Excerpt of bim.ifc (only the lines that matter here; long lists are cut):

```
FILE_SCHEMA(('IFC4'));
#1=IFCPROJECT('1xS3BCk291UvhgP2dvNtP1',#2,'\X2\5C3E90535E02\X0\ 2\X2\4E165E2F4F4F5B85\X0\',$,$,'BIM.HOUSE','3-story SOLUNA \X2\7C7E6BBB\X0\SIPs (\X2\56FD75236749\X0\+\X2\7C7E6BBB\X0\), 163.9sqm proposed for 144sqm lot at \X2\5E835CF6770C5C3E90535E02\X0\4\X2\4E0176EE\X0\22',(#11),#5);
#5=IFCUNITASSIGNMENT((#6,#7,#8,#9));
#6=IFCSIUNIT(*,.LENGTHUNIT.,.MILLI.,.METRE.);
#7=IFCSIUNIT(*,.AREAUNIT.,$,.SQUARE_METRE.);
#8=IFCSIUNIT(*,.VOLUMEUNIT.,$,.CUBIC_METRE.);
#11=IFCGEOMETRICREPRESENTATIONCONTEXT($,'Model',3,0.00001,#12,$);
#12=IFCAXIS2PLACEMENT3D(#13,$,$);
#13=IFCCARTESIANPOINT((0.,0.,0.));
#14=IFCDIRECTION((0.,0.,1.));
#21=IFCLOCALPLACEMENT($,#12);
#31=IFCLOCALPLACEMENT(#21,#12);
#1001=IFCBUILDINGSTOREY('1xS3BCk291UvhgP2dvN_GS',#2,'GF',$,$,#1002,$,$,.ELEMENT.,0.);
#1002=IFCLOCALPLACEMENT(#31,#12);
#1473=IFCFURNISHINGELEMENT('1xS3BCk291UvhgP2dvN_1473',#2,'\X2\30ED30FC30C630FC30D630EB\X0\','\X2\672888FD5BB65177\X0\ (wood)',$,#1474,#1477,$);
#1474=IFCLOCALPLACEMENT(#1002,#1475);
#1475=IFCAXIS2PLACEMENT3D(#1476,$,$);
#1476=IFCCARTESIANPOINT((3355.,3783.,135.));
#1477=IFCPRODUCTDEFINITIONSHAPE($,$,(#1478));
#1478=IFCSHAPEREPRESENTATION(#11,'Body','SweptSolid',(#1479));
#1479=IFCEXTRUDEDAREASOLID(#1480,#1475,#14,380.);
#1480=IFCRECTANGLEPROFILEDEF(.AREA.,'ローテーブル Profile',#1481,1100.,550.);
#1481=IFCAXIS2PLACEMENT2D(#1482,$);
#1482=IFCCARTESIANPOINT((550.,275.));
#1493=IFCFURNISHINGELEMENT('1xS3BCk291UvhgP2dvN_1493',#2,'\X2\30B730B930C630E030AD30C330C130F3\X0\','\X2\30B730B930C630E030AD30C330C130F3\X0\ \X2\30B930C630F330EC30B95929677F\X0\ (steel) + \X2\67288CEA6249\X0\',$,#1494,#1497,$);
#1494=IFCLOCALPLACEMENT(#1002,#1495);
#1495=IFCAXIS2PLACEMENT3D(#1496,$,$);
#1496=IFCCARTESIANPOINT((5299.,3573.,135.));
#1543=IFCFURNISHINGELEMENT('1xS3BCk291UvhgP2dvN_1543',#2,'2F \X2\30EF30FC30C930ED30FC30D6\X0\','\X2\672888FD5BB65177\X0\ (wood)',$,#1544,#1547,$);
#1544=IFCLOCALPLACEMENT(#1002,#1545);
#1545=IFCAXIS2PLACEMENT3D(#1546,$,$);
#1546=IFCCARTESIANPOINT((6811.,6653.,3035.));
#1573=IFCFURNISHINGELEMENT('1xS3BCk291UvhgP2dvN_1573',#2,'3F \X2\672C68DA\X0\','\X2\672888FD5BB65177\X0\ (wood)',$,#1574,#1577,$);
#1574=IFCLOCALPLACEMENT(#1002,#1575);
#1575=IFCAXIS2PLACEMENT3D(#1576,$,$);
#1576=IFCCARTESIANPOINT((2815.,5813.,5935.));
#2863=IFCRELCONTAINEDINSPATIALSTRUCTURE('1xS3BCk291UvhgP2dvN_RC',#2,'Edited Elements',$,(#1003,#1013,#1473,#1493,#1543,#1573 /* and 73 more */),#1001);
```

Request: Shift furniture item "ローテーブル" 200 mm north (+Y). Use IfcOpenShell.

```python
import ifcopenshell
import ifcopenshell.api.geometry
import ifcopenshell.util.placement
import ifcopenshell.util.unit

model = ifcopenshell.open("bim.ifc")
unit_scale = ifcopenshell.util.unit.calculate_unit_scale(model)

item = model.by_guid("1xS3BCk291UvhgP2dvN_1473")
matrix = ifcopenshell.util.placement.get_local_placement(item.ObjectPlacement)
matrix[1, 3] += 0.2 / unit_scale
ifcopenshell.api.geometry.edit_object_placement(model, product=item, matrix=matrix, is_si=False)

print(ifcopenshell.util.placement.get_local_placement(item.ObjectPlacement).round(3) + 0.0)

model.write("bim_rev.ifc")
```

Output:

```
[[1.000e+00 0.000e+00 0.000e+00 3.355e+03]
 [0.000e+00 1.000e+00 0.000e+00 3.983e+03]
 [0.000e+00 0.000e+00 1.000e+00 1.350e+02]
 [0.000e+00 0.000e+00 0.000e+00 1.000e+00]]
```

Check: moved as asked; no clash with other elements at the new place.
